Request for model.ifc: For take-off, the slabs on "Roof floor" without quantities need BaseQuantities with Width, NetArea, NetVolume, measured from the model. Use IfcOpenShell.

First a look at what the model holds.

```python
import ifcopenshell
import ifcopenshell.util.element
import ifcopenshell.util.unit

model = ifcopenshell.open("model.ifc")
print(model.schema)
for unit_type in ("LENGTHUNIT", "AREAUNIT", "VOLUMEUNIT"):
    print(unit_type, ifcopenshell.util.unit.calculate_unit_scale(model, unit_type))
storey = next(s for s in model.by_type("IfcBuildingStorey") if s.Name == "Roof floor")
slabs = [e for e in ifcopenshell.util.element.get_decomposition(storey) if e.is_a("IfcSlab")]
for e in sorted(slabs, key=lambda e: e.id()):
    print(e.id(), e.is_a(), e.Name, list(ifcopenshell.util.element.get_psets(e, qtos_only=True)), sep=" | ")
```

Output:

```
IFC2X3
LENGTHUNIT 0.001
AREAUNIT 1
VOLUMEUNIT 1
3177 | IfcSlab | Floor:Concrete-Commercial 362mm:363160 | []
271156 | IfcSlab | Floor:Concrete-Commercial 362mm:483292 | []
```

```python
import ifcopenshell
import ifcopenshell.api.pset
import ifcopenshell.geom
import ifcopenshell.util.element
import ifcopenshell.util.shape
import ifcopenshell.util.unit

model = ifcopenshell.open("model.ifc")
unit_scale = ifcopenshell.util.unit.calculate_unit_scale(model)
area_scale = ifcopenshell.util.unit.calculate_unit_scale(model, "AREAUNIT")
volume_scale = ifcopenshell.util.unit.calculate_unit_scale(model, "VOLUMEUNIT")
settings = ifcopenshell.geom.settings()

storey = next(s for s in model.by_type("IfcBuildingStorey") if s.Name == "Roof floor")
slabs = [e for e in ifcopenshell.util.element.get_decomposition(storey) if e.is_a("IfcSlab")]

for e in sorted(slabs, key=lambda e: e.id()):
    if ifcopenshell.util.element.get_psets(e, qtos_only=True, should_inherit=False):
        continue
    # Geometry comes back in metres, in the element's own axes.
    shape = ifcopenshell.geom.create_shape(settings, e)
    values = {
        "Width": ifcopenshell.util.shape.get_z(shape.geometry) / unit_scale,
        "NetArea": ifcopenshell.util.shape.get_footprint_area(shape.geometry) / area_scale,
        "NetVolume": ifcopenshell.util.shape.get_volume(shape.geometry) / volume_scale,
    }
    qto = ifcopenshell.api.pset.add_qto(model, product=e, name="BaseQuantities")
    ifcopenshell.api.pset.edit_qto(model, qto=qto, properties=values)
    print(e.id(), {k: round(v, 3) for k, v in values.items()})

model.write("model_rev.ifc")
```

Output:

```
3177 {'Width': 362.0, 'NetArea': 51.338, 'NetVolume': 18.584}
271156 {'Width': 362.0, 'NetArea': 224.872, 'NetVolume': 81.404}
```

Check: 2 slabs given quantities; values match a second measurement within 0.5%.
